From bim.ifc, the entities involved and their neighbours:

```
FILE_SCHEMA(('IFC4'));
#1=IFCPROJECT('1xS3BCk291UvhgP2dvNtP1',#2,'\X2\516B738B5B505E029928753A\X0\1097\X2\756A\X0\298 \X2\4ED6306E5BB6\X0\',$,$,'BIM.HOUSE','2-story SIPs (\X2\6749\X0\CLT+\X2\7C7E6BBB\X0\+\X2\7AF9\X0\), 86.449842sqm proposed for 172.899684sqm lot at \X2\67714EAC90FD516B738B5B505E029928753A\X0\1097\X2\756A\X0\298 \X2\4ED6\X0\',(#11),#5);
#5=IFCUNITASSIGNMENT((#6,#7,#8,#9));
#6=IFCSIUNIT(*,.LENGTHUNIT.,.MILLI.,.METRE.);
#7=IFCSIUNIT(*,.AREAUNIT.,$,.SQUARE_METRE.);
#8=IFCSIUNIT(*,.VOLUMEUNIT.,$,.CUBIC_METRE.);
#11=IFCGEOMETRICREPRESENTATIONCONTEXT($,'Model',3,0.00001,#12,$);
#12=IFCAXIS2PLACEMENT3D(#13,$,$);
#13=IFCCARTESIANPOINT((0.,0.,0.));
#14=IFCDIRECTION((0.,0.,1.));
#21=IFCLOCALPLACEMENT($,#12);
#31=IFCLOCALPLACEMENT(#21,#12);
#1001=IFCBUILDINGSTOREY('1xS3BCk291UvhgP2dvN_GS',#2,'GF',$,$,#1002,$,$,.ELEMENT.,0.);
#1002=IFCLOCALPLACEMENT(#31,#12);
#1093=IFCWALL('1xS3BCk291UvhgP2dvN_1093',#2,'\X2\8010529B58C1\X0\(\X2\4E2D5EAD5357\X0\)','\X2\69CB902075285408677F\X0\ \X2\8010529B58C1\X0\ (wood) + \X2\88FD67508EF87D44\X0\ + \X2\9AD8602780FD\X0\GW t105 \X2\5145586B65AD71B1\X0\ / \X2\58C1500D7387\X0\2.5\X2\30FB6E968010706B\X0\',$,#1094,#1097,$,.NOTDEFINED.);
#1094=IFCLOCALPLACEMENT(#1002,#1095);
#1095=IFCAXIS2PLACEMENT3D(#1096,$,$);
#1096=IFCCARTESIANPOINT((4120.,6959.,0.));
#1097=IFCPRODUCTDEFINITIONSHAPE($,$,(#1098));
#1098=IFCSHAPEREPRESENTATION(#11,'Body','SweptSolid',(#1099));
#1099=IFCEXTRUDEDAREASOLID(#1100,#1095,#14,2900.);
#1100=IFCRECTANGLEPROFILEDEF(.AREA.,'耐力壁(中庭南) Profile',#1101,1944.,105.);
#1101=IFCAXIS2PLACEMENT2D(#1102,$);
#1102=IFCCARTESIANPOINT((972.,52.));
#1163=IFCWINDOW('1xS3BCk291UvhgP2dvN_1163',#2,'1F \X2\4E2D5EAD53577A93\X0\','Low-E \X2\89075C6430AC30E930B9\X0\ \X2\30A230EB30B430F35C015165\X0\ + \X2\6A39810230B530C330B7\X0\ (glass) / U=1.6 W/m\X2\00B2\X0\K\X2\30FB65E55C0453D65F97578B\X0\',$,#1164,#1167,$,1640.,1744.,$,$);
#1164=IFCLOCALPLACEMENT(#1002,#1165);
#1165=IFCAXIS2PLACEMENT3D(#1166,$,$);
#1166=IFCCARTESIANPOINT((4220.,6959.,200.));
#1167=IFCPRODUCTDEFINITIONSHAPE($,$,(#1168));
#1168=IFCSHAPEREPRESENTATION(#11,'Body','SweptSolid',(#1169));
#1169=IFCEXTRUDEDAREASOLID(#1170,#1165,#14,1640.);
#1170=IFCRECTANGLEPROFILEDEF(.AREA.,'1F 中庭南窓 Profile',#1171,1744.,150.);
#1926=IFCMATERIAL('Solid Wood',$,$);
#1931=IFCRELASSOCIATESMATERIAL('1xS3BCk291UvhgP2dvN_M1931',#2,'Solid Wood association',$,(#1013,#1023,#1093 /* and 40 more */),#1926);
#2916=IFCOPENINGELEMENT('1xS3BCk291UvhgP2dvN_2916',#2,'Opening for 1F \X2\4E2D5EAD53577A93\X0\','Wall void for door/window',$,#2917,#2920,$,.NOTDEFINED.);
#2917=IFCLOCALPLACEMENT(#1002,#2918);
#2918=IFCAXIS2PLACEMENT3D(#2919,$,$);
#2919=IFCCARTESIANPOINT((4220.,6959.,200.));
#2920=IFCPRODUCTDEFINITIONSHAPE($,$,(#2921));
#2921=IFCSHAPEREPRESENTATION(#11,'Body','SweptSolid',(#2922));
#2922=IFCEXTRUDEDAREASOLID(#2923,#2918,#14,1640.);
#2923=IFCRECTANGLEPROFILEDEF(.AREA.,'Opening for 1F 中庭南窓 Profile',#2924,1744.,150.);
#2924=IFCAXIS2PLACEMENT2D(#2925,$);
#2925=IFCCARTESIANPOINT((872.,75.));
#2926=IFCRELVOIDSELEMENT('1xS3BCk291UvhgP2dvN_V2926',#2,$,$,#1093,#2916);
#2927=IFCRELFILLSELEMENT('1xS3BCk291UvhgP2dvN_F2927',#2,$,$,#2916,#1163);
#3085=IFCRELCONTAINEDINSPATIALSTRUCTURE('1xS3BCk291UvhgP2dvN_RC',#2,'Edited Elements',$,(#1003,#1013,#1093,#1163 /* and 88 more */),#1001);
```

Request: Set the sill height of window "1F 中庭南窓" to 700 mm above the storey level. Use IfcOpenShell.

```python
import numpy as np
import ifcopenshell
import ifcopenshell.api.geometry
import ifcopenshell.geom
import ifcopenshell.util.element
import ifcopenshell.util.placement
import ifcopenshell.util.shape
import ifcopenshell.util.unit

model = ifcopenshell.open("bim.ifc")
unit_scale = ifcopenshell.util.unit.calculate_unit_scale(model)

window = model.by_id(1163)
opening = window.FillsVoids[0].RelatingOpeningElement
storey = ifcopenshell.util.element.get_container(window, ifc_class="IfcBuildingStorey")
level = ifcopenshell.util.placement.get_local_placement(storey.ObjectPlacement)[2, 3]

# The opening's origin need not be at the sill, so measure its lowest point.
shape = ifcopenshell.geom.create_shape(ifcopenshell.geom.settings(), opening)
bottom = ifcopenshell.util.shape.get_shape_bottom_elevation(shape, shape.geometry) / unit_scale
dz = level + 0.7 / unit_scale - bottom

shift = np.array([0.0, 0.0, dz])
# The window is not placed relative to its opening, so move both.
for product in (opening, window):
    matrix = ifcopenshell.util.placement.get_local_placement(product.ObjectPlacement)
    matrix[:3, 3] += shift
    ifcopenshell.api.geometry.edit_object_placement(model, product=product, matrix=matrix, is_si=False)

print(f"moved by {dz * unit_scale:+.3f} m")

model.write("bim_v2.ifc")
```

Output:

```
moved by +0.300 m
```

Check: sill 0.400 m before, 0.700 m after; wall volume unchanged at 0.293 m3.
